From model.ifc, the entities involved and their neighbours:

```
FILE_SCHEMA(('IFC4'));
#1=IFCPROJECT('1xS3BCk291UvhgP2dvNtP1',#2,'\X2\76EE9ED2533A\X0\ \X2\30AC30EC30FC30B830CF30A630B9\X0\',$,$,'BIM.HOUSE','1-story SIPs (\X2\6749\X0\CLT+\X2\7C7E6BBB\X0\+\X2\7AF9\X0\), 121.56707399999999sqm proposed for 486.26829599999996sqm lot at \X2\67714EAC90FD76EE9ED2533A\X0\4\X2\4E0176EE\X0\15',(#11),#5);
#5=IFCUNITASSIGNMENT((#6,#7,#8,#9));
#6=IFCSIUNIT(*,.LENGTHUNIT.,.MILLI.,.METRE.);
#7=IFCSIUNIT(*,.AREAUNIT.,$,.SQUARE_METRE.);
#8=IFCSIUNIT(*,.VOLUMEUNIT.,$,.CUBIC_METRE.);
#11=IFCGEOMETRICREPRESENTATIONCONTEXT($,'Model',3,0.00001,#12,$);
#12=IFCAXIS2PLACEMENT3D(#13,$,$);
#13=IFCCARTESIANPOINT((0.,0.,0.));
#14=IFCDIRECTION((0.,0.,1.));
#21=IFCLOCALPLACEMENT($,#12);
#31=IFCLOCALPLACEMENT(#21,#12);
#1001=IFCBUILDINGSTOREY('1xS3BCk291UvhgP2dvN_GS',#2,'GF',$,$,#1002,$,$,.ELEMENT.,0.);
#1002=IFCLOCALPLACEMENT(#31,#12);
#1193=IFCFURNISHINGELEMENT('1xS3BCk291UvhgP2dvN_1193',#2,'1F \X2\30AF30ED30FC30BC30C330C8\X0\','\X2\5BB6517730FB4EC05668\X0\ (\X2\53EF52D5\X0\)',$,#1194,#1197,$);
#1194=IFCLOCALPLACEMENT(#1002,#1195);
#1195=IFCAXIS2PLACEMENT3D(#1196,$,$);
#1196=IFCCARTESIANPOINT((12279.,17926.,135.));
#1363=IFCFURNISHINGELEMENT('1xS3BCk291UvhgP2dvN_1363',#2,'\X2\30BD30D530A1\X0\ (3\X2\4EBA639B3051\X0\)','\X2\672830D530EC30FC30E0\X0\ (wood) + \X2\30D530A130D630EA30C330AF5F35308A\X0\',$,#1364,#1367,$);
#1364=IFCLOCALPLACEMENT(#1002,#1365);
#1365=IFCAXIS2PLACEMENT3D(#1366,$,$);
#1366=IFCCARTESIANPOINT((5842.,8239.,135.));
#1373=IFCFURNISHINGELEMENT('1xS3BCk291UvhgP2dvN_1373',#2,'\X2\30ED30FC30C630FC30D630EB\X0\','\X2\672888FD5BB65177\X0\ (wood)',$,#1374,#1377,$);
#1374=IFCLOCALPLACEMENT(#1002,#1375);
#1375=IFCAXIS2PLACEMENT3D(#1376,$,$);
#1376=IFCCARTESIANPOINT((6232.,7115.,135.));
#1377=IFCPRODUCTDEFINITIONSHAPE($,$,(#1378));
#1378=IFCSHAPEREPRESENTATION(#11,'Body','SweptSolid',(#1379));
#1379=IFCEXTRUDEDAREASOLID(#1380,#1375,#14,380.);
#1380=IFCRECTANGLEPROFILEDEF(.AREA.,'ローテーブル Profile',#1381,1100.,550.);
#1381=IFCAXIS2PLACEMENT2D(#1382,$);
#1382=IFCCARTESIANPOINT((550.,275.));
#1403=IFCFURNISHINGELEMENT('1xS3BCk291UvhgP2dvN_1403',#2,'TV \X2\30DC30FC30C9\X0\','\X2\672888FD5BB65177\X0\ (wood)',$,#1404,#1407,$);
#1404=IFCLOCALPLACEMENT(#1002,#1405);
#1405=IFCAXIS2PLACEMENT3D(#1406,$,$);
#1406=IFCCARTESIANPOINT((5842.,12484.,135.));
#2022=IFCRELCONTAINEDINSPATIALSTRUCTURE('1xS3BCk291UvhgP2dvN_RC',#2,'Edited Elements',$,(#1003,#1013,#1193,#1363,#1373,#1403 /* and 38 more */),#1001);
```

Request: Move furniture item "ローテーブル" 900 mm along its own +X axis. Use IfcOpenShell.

```python
import ifcopenshell
import ifcopenshell.api.geometry
import ifcopenshell.util.placement

model = ifcopenshell.open("model.ifc")

item = model.by_guid("1xS3BCk291UvhgP2dvN_1373")
matrix = ifcopenshell.util.placement.get_local_placement(item.ObjectPlacement)
matrix[:3, 3] += matrix[:3, 0] * 900.0
ifcopenshell.api.geometry.edit_object_placement(model, product=item, matrix=matrix, is_si=False)

print(ifcopenshell.util.placement.get_local_placement(item.ObjectPlacement).round(3) + 0.0)

model.write("model_edited.ifc")
```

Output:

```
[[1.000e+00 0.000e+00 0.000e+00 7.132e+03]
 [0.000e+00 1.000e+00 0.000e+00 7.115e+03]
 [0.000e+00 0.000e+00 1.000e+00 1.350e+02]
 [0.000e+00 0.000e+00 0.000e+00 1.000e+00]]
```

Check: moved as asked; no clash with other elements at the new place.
